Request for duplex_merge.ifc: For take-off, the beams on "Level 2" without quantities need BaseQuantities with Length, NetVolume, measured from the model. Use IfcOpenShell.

First a look at what the model holds.

```python
import ifcopenshell
import ifcopenshell.util.element
import ifcopenshell.util.unit

model = ifcopenshell.open("duplex_merge.ifc")
print(model.schema)
for unit_type in ("LENGTHUNIT", "AREAUNIT", "VOLUMEUNIT"):
    print(unit_type, ifcopenshell.util.unit.calculate_unit_scale(model, unit_type))
storey = next(s for s in model.by_type("IfcBuildingStorey") if s.Name == "Level 2")
beams = [e for e in ifcopenshell.util.element.get_decomposition(storey) if e.is_a("IfcBeam")]
for e in sorted(beams, key=lambda e: e.id()):
    print(e.id(), e.is_a(), e.Name, list(ifcopenshell.util.element.get_psets(e, qtos_only=True)), sep=" | ")
```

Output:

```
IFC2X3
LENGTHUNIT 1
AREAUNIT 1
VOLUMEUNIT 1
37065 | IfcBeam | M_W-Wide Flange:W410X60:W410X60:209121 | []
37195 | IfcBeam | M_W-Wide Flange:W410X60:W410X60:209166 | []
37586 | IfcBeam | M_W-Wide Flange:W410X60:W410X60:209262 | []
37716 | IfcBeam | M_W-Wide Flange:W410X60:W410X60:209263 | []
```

```python
import ifcopenshell
import ifcopenshell.api.pset
import ifcopenshell.geom
import ifcopenshell.util.element
import ifcopenshell.util.shape
import ifcopenshell.util.unit

model = ifcopenshell.open("duplex_merge.ifc")
unit_scale = ifcopenshell.util.unit.calculate_unit_scale(model)
volume_scale = ifcopenshell.util.unit.calculate_unit_scale(model, "VOLUMEUNIT")
settings = ifcopenshell.geom.settings()

storey = next(s for s in model.by_type("IfcBuildingStorey") if s.Name == "Level 2")
beams = [e for e in ifcopenshell.util.element.get_decomposition(storey) if e.is_a("IfcBeam")]

for e in sorted(beams, key=lambda e: e.id()):
    if ifcopenshell.util.element.get_psets(e, qtos_only=True, should_inherit=False):
        continue
    # Geometry comes back in metres, in the element's own axes.
    shape = ifcopenshell.geom.create_shape(settings, e)
    values = {
        "Length": ifcopenshell.util.shape.get_max_xyz(shape.geometry) / unit_scale,
        "NetVolume": ifcopenshell.util.shape.get_volume(shape.geometry) / volume_scale,
    }
    qto = ifcopenshell.api.pset.add_qto(model, product=e, name="BaseQuantities")
    ifcopenshell.api.pset.edit_qto(model, qto=qto, properties=values)
    print(e.id(), {k: round(v, 3) for k, v in values.items()})

model.write("duplex_merge_rev.ifc")
```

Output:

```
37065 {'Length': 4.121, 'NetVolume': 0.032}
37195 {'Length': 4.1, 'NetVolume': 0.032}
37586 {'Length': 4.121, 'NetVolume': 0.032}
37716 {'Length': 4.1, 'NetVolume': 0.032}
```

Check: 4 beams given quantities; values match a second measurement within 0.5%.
